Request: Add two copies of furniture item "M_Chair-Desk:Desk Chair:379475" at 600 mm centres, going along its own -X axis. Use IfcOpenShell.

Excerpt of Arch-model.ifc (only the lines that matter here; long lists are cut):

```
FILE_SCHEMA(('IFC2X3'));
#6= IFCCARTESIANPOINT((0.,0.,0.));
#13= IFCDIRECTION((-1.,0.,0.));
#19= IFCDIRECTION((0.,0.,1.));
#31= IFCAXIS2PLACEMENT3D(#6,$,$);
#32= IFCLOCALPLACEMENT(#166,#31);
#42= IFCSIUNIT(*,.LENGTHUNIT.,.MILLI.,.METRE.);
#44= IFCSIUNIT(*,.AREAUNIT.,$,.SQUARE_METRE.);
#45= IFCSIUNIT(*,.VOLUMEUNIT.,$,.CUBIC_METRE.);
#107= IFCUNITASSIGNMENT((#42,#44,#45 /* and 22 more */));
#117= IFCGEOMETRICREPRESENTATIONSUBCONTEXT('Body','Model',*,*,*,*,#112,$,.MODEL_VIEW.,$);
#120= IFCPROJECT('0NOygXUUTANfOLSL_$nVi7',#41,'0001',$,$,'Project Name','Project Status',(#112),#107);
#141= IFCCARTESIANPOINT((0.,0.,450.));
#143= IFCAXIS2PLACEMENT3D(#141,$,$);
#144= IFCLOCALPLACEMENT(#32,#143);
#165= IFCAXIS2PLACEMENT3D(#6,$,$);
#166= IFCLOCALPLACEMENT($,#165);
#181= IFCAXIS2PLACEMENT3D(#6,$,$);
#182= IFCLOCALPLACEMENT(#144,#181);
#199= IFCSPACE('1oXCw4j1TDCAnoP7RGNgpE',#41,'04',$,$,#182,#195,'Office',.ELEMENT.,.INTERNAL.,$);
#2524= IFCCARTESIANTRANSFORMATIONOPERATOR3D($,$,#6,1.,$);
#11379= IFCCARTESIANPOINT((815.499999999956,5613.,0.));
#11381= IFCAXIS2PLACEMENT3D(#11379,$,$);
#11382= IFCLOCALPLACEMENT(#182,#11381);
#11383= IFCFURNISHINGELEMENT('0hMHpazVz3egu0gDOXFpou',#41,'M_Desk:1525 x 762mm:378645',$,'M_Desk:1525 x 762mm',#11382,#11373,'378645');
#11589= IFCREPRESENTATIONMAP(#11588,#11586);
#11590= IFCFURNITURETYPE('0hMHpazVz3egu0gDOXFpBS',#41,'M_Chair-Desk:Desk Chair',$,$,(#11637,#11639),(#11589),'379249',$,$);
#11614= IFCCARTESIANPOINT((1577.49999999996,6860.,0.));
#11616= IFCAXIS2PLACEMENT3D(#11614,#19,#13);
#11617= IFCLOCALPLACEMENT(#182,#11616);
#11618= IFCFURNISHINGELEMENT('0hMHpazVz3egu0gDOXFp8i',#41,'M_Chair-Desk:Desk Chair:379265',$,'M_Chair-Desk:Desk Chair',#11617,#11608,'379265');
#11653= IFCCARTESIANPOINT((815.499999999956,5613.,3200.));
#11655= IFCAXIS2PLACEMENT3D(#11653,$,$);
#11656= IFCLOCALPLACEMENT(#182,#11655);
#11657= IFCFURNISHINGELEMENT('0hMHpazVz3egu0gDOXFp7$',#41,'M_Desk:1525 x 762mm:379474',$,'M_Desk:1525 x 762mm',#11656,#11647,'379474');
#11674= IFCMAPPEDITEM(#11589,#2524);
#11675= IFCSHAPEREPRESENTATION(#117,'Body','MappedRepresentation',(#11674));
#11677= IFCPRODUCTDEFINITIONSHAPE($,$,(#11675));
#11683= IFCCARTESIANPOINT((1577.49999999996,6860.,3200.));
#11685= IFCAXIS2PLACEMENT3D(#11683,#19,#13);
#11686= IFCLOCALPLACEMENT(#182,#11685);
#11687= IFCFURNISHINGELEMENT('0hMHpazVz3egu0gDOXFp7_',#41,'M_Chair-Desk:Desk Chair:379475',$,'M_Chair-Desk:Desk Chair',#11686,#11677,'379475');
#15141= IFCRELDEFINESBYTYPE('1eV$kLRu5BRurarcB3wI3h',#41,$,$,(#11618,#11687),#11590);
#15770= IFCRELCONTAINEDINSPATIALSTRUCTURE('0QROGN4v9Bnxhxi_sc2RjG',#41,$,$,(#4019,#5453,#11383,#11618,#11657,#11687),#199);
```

```python
import ifcopenshell
import ifcopenshell.api.geometry
import ifcopenshell.api.root
import ifcopenshell.util.element
import ifcopenshell.util.placement
import ifcopenshell.util.unit

model = ifcopenshell.open("Arch-model.ifc")
unit_scale = ifcopenshell.util.unit.calculate_unit_scale(model)


def reuse_history(source, copy):
    """copy_class also copies each property set's owner history, people and application; keep the originals."""
    for rel in copy.IsDefinedBy:
        if rel.is_a("IfcRelDefinesByProperties") and (history := rel.RelatingPropertyDefinition.OwnerHistory):
            rel.RelatingPropertyDefinition.OwnerHistory = source.OwnerHistory
            ifcopenshell.util.element.remove_deep2(model, history)


source = model.by_id(11687)
base = ifcopenshell.util.placement.get_local_placement(source.ObjectPlacement)
step = -base[:3, 0] * 0.6 / unit_scale

for i in range(1, 3):
    copy = ifcopenshell.api.root.copy_class(model, product=source)
    copy.Representation = ifcopenshell.util.element.copy_deep(
        model, source.Representation, exclude=["IfcGeometricRepresentationContext", "IfcRepresentationMap"]
    )
    copy.Name = "M_Chair-Desk:Desk Chair"
    copy.Tag = None
    reuse_history(source, copy)
    matrix = base.copy()
    matrix[:3, 3] += i * step
    print("added at", matrix[:3, 3].round(3) + 0.0)
    ifcopenshell.api.geometry.edit_object_placement(model, product=copy, matrix=matrix, is_si=False)

model.write("Arch-model-out.ifc")
```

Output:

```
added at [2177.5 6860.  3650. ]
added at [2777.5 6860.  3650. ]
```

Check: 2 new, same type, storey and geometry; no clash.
